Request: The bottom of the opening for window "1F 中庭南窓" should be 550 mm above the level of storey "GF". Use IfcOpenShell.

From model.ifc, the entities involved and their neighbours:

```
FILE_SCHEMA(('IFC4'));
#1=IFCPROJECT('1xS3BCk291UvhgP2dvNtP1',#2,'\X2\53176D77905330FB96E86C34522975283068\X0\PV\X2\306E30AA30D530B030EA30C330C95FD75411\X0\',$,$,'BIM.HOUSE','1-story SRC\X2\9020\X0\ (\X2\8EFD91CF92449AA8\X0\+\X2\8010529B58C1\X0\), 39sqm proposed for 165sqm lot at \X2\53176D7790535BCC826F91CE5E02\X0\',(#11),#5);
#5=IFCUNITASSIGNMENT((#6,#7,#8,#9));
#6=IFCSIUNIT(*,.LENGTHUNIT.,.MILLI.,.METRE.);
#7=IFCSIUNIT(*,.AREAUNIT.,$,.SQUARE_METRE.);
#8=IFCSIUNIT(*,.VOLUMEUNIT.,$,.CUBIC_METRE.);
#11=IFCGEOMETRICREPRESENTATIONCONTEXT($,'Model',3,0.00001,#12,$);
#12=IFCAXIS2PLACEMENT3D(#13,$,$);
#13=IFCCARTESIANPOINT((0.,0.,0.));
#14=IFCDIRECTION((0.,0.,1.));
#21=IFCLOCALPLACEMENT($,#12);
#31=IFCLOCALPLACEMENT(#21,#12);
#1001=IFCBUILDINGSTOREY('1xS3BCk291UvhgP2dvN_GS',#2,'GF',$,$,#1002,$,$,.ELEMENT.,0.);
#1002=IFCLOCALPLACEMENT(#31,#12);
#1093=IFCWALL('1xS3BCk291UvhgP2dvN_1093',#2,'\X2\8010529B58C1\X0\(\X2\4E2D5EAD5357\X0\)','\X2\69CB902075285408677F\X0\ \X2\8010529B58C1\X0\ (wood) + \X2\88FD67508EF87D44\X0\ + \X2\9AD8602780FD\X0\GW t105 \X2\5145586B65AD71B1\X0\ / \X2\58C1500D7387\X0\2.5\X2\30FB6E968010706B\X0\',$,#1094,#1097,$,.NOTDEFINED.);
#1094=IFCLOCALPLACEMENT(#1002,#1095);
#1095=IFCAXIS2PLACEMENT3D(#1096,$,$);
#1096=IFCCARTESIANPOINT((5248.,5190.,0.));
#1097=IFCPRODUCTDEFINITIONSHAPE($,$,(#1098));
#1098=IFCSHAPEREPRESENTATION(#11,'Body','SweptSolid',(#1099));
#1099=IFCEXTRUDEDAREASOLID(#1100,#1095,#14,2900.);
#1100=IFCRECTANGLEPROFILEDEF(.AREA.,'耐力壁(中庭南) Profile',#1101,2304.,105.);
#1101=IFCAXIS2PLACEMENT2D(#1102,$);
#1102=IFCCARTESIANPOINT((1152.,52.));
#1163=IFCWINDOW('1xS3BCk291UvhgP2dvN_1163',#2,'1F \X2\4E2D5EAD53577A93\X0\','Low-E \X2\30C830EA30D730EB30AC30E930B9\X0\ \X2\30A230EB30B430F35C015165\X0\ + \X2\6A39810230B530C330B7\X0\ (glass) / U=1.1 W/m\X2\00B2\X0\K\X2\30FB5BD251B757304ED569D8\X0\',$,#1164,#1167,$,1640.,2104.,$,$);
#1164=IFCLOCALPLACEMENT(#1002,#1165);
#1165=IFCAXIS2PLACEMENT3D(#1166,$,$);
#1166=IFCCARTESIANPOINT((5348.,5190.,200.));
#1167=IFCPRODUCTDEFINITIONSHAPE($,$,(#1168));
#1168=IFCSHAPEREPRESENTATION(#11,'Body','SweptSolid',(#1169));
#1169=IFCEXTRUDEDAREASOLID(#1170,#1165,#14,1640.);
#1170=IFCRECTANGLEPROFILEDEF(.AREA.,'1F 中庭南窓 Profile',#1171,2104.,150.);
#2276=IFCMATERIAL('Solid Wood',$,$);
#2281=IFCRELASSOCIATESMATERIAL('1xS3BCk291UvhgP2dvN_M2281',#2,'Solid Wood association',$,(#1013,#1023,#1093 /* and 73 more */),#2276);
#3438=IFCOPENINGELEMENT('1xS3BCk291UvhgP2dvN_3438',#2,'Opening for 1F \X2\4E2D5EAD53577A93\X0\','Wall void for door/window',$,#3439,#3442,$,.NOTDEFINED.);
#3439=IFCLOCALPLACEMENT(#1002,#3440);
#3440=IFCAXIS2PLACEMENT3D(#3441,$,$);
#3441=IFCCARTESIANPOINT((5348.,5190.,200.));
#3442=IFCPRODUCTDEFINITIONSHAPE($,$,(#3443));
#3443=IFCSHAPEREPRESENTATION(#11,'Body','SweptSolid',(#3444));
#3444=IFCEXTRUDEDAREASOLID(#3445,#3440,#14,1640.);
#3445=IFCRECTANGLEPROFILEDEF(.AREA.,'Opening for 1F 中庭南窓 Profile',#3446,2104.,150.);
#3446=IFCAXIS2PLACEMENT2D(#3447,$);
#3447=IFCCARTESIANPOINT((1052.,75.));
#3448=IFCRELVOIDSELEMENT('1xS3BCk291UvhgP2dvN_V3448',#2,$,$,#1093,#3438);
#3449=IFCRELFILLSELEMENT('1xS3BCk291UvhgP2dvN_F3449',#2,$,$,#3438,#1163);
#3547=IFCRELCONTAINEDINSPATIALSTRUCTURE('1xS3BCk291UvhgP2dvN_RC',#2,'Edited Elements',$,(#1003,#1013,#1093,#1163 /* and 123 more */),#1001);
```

```python
import numpy as np
import ifcopenshell
import ifcopenshell.api.geometry
import ifcopenshell.geom
import ifcopenshell.util.element
import ifcopenshell.util.placement
import ifcopenshell.util.shape
import ifcopenshell.util.unit

model = ifcopenshell.open("model.ifc")
unit_scale = ifcopenshell.util.unit.calculate_unit_scale(model)

window = model.by_guid("1xS3BCk291UvhgP2dvN_1163")
opening = window.FillsVoids[0].RelatingOpeningElement
storey = ifcopenshell.util.element.get_container(window, ifc_class="IfcBuildingStorey")
level = ifcopenshell.util.placement.get_local_placement(storey.ObjectPlacement)[2, 3]

# The opening's origin need not be at the sill, so measure its lowest point.
shape = ifcopenshell.geom.create_shape(ifcopenshell.geom.settings(), opening)
bottom = ifcopenshell.util.shape.get_shape_bottom_elevation(shape, shape.geometry) / unit_scale
dz = level + 0.55 / unit_scale - bottom

shift = np.array([0.0, 0.0, dz])
# The window is not placed relative to its opening, so move both.
for product in (opening, window):
    matrix = ifcopenshell.util.placement.get_local_placement(product.ObjectPlacement)
    matrix[:3, 3] += shift
    ifcopenshell.api.geometry.edit_object_placement(model, product=product, matrix=matrix, is_si=False)

print(f"moved by {dz * unit_scale:+.3f} m")

model.write("model_edited.ifc")
```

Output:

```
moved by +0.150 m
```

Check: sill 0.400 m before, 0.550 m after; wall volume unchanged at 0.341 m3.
